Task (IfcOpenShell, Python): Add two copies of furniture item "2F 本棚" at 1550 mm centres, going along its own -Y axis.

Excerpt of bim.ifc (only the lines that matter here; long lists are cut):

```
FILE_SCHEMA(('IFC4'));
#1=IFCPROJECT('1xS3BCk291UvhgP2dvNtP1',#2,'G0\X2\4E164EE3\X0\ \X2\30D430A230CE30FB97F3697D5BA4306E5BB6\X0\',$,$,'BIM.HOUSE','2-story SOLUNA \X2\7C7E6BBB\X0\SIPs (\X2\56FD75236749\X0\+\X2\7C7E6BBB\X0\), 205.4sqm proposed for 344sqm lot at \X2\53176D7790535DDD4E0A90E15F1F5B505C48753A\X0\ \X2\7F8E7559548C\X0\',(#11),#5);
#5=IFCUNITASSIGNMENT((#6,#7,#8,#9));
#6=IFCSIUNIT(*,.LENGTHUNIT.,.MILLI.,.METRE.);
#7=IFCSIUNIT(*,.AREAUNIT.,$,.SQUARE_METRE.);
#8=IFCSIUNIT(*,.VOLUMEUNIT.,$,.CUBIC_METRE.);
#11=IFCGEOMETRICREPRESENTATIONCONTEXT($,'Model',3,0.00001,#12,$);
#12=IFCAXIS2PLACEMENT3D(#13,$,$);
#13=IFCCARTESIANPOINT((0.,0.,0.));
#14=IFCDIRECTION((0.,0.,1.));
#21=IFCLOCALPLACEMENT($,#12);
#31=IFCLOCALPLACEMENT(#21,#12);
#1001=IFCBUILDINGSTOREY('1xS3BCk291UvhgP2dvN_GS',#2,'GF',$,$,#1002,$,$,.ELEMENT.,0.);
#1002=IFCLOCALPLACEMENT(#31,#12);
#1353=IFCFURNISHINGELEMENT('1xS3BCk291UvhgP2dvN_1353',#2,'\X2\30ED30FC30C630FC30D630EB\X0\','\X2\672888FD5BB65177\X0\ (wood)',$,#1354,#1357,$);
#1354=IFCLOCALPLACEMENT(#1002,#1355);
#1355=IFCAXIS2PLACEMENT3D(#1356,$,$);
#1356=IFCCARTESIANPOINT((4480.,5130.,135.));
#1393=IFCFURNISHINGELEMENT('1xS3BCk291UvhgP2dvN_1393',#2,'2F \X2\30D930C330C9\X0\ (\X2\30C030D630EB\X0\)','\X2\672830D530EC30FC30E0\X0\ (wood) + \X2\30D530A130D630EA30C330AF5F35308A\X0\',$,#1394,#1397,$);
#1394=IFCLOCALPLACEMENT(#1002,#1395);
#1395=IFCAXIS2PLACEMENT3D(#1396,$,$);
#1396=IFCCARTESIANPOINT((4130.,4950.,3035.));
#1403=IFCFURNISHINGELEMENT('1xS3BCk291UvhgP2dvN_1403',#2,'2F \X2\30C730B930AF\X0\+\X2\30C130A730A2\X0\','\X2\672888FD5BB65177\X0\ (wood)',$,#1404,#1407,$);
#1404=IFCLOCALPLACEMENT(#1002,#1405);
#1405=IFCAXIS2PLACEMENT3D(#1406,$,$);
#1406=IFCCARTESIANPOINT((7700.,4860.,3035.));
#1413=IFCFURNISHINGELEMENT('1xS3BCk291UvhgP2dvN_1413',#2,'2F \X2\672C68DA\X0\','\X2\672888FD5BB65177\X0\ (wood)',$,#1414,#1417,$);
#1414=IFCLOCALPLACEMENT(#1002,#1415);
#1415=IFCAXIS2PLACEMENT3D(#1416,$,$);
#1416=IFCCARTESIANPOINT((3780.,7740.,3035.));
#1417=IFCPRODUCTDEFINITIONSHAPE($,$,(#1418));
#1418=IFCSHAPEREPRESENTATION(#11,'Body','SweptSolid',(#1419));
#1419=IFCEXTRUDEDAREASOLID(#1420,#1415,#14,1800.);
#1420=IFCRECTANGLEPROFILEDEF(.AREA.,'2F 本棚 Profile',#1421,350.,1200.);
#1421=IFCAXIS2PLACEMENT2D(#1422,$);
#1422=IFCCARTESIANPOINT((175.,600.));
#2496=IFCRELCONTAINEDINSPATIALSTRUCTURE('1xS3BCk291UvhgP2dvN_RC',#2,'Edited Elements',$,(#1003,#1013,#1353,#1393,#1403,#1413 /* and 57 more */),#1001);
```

```python
import ifcopenshell
import ifcopenshell.api.geometry
import ifcopenshell.api.root
import ifcopenshell.util.element
import ifcopenshell.util.placement
import ifcopenshell.util.unit

model = ifcopenshell.open("bim.ifc")
unit_scale = ifcopenshell.util.unit.calculate_unit_scale(model)


def reuse_history(source, copy):
    """copy_class also copies each property set's owner history, people and application; keep the originals."""
    for rel in copy.IsDefinedBy:
        if rel.is_a("IfcRelDefinesByProperties") and (history := rel.RelatingPropertyDefinition.OwnerHistory):
            rel.RelatingPropertyDefinition.OwnerHistory = source.OwnerHistory
            ifcopenshell.util.element.remove_deep2(model, history)


source = model.by_guid("1xS3BCk291UvhgP2dvN_1413")
base = ifcopenshell.util.placement.get_local_placement(source.ObjectPlacement)
step = -base[:3, 1] * 1.55 / unit_scale

for i in range(1, 3):
    copy = ifcopenshell.api.root.copy_class(model, product=source)
    copy.Representation = ifcopenshell.util.element.copy_deep(
        model, source.Representation, exclude=["IfcGeometricRepresentationContext", "IfcRepresentationMap"]
    )
    reuse_history(source, copy)
    matrix = base.copy()
    matrix[:3, 3] += i * step
    print("added at", matrix[:3, 3].round(3) + 0.0)
    ifcopenshell.api.geometry.edit_object_placement(model, product=copy, matrix=matrix, is_si=False)

model.write("bim_rev.ifc")
```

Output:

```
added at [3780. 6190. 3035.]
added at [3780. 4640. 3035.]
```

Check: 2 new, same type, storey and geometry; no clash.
